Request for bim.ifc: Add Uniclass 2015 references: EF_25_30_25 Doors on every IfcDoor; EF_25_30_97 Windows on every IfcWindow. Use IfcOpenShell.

First a look at what the model holds.

```python
import ifcopenshell

model = ifcopenshell.open("bim.ifc")
print(model.schema)
print("classifications:", [c.Name for c in model.by_type("IfcClassification")])
for ifc_class in ("IfcDoor", "IfcRoof", "IfcStair", "IfcWall", "IfcWindow"):
    print(ifc_class, len(model.by_type(ifc_class)))
```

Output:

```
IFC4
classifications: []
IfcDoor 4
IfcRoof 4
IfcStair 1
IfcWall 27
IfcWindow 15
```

```python
import ifcopenshell
import ifcopenshell.api.classification

model = ifcopenshell.open("bim.ifc")

system = ifcopenshell.api.classification.add_classification(model, classification="Uniclass 2015")

codes = {
    "IfcDoor": ("EF_25_30_25", "Doors"),
    "IfcWindow": ("EF_25_30_97", "Windows"),
}
for ifc_class, (code, name) in codes.items():
    products = model.by_type(ifc_class)
    ifcopenshell.api.classification.add_reference(
        model, products=products, classification=system, identification=code, name=name
    )
    print(code, len(products))

model.write("bim-out.ifc")
```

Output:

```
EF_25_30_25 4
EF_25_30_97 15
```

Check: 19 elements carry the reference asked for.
